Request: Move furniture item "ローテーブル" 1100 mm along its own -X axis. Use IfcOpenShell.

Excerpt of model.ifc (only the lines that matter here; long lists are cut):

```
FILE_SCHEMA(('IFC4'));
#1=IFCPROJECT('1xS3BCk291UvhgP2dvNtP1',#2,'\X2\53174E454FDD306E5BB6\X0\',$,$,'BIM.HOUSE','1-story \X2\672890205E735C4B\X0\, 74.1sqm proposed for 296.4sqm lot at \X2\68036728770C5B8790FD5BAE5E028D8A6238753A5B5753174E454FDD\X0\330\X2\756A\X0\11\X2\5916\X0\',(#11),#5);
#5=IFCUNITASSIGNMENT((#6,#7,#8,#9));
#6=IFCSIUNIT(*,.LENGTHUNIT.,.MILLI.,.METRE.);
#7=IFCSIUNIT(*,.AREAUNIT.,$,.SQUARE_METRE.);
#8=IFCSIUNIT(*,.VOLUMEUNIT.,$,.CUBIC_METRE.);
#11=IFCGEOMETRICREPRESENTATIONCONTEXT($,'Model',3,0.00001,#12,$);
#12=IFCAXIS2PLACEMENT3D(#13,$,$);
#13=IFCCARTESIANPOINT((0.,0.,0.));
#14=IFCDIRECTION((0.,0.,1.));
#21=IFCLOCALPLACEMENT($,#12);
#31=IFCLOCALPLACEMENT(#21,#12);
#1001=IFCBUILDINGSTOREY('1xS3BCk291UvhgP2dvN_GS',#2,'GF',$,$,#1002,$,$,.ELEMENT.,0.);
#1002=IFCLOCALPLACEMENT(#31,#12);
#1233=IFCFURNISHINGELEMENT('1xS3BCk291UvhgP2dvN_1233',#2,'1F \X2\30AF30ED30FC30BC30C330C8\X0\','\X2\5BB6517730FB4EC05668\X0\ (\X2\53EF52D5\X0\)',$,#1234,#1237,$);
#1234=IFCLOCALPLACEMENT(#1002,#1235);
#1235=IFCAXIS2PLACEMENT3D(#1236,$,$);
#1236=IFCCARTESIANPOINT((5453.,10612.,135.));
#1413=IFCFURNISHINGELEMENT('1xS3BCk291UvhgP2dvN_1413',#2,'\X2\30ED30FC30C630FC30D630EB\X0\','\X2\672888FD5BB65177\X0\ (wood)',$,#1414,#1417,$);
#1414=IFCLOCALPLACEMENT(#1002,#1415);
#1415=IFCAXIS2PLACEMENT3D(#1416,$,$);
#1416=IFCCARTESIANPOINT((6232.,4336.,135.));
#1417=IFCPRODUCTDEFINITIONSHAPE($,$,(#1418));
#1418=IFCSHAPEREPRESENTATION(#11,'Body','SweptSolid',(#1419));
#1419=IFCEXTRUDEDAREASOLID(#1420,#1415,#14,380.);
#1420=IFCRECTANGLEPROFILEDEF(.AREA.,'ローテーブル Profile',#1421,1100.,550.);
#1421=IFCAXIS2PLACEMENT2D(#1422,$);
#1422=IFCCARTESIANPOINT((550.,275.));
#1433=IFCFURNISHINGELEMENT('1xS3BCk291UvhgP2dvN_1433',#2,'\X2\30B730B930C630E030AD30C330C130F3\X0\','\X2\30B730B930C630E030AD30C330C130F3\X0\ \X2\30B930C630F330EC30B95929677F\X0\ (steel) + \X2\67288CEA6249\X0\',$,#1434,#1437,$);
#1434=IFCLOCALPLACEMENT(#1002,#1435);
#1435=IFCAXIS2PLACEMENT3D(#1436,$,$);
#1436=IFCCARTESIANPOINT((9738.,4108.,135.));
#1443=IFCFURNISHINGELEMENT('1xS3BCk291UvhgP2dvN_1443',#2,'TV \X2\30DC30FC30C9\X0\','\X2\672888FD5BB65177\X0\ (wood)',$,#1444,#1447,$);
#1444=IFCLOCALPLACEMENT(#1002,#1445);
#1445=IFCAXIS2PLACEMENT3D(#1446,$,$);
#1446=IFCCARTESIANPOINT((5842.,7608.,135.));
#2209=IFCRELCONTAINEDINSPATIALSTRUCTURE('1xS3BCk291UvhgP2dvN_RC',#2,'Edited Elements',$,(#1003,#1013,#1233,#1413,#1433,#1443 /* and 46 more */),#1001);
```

```python
import ifcopenshell
import ifcopenshell.api.geometry
import ifcopenshell.util.placement
import ifcopenshell.util.unit

model = ifcopenshell.open("model.ifc")
unit_scale = ifcopenshell.util.unit.calculate_unit_scale(model)

item = model.by_id(1413)
matrix = ifcopenshell.util.placement.get_local_placement(item.ObjectPlacement)
matrix[:3, 3] -= matrix[:3, 0] * 1.1 / unit_scale
ifcopenshell.api.geometry.edit_object_placement(model, product=item, matrix=matrix, is_si=False)

print(ifcopenshell.util.placement.get_local_placement(item.ObjectPlacement).round(3) + 0.0)

model.write("model_v2.ifc")
```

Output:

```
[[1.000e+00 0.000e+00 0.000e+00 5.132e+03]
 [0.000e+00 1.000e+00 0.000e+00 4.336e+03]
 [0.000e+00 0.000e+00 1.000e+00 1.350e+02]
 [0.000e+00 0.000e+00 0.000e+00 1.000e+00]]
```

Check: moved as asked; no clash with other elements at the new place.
